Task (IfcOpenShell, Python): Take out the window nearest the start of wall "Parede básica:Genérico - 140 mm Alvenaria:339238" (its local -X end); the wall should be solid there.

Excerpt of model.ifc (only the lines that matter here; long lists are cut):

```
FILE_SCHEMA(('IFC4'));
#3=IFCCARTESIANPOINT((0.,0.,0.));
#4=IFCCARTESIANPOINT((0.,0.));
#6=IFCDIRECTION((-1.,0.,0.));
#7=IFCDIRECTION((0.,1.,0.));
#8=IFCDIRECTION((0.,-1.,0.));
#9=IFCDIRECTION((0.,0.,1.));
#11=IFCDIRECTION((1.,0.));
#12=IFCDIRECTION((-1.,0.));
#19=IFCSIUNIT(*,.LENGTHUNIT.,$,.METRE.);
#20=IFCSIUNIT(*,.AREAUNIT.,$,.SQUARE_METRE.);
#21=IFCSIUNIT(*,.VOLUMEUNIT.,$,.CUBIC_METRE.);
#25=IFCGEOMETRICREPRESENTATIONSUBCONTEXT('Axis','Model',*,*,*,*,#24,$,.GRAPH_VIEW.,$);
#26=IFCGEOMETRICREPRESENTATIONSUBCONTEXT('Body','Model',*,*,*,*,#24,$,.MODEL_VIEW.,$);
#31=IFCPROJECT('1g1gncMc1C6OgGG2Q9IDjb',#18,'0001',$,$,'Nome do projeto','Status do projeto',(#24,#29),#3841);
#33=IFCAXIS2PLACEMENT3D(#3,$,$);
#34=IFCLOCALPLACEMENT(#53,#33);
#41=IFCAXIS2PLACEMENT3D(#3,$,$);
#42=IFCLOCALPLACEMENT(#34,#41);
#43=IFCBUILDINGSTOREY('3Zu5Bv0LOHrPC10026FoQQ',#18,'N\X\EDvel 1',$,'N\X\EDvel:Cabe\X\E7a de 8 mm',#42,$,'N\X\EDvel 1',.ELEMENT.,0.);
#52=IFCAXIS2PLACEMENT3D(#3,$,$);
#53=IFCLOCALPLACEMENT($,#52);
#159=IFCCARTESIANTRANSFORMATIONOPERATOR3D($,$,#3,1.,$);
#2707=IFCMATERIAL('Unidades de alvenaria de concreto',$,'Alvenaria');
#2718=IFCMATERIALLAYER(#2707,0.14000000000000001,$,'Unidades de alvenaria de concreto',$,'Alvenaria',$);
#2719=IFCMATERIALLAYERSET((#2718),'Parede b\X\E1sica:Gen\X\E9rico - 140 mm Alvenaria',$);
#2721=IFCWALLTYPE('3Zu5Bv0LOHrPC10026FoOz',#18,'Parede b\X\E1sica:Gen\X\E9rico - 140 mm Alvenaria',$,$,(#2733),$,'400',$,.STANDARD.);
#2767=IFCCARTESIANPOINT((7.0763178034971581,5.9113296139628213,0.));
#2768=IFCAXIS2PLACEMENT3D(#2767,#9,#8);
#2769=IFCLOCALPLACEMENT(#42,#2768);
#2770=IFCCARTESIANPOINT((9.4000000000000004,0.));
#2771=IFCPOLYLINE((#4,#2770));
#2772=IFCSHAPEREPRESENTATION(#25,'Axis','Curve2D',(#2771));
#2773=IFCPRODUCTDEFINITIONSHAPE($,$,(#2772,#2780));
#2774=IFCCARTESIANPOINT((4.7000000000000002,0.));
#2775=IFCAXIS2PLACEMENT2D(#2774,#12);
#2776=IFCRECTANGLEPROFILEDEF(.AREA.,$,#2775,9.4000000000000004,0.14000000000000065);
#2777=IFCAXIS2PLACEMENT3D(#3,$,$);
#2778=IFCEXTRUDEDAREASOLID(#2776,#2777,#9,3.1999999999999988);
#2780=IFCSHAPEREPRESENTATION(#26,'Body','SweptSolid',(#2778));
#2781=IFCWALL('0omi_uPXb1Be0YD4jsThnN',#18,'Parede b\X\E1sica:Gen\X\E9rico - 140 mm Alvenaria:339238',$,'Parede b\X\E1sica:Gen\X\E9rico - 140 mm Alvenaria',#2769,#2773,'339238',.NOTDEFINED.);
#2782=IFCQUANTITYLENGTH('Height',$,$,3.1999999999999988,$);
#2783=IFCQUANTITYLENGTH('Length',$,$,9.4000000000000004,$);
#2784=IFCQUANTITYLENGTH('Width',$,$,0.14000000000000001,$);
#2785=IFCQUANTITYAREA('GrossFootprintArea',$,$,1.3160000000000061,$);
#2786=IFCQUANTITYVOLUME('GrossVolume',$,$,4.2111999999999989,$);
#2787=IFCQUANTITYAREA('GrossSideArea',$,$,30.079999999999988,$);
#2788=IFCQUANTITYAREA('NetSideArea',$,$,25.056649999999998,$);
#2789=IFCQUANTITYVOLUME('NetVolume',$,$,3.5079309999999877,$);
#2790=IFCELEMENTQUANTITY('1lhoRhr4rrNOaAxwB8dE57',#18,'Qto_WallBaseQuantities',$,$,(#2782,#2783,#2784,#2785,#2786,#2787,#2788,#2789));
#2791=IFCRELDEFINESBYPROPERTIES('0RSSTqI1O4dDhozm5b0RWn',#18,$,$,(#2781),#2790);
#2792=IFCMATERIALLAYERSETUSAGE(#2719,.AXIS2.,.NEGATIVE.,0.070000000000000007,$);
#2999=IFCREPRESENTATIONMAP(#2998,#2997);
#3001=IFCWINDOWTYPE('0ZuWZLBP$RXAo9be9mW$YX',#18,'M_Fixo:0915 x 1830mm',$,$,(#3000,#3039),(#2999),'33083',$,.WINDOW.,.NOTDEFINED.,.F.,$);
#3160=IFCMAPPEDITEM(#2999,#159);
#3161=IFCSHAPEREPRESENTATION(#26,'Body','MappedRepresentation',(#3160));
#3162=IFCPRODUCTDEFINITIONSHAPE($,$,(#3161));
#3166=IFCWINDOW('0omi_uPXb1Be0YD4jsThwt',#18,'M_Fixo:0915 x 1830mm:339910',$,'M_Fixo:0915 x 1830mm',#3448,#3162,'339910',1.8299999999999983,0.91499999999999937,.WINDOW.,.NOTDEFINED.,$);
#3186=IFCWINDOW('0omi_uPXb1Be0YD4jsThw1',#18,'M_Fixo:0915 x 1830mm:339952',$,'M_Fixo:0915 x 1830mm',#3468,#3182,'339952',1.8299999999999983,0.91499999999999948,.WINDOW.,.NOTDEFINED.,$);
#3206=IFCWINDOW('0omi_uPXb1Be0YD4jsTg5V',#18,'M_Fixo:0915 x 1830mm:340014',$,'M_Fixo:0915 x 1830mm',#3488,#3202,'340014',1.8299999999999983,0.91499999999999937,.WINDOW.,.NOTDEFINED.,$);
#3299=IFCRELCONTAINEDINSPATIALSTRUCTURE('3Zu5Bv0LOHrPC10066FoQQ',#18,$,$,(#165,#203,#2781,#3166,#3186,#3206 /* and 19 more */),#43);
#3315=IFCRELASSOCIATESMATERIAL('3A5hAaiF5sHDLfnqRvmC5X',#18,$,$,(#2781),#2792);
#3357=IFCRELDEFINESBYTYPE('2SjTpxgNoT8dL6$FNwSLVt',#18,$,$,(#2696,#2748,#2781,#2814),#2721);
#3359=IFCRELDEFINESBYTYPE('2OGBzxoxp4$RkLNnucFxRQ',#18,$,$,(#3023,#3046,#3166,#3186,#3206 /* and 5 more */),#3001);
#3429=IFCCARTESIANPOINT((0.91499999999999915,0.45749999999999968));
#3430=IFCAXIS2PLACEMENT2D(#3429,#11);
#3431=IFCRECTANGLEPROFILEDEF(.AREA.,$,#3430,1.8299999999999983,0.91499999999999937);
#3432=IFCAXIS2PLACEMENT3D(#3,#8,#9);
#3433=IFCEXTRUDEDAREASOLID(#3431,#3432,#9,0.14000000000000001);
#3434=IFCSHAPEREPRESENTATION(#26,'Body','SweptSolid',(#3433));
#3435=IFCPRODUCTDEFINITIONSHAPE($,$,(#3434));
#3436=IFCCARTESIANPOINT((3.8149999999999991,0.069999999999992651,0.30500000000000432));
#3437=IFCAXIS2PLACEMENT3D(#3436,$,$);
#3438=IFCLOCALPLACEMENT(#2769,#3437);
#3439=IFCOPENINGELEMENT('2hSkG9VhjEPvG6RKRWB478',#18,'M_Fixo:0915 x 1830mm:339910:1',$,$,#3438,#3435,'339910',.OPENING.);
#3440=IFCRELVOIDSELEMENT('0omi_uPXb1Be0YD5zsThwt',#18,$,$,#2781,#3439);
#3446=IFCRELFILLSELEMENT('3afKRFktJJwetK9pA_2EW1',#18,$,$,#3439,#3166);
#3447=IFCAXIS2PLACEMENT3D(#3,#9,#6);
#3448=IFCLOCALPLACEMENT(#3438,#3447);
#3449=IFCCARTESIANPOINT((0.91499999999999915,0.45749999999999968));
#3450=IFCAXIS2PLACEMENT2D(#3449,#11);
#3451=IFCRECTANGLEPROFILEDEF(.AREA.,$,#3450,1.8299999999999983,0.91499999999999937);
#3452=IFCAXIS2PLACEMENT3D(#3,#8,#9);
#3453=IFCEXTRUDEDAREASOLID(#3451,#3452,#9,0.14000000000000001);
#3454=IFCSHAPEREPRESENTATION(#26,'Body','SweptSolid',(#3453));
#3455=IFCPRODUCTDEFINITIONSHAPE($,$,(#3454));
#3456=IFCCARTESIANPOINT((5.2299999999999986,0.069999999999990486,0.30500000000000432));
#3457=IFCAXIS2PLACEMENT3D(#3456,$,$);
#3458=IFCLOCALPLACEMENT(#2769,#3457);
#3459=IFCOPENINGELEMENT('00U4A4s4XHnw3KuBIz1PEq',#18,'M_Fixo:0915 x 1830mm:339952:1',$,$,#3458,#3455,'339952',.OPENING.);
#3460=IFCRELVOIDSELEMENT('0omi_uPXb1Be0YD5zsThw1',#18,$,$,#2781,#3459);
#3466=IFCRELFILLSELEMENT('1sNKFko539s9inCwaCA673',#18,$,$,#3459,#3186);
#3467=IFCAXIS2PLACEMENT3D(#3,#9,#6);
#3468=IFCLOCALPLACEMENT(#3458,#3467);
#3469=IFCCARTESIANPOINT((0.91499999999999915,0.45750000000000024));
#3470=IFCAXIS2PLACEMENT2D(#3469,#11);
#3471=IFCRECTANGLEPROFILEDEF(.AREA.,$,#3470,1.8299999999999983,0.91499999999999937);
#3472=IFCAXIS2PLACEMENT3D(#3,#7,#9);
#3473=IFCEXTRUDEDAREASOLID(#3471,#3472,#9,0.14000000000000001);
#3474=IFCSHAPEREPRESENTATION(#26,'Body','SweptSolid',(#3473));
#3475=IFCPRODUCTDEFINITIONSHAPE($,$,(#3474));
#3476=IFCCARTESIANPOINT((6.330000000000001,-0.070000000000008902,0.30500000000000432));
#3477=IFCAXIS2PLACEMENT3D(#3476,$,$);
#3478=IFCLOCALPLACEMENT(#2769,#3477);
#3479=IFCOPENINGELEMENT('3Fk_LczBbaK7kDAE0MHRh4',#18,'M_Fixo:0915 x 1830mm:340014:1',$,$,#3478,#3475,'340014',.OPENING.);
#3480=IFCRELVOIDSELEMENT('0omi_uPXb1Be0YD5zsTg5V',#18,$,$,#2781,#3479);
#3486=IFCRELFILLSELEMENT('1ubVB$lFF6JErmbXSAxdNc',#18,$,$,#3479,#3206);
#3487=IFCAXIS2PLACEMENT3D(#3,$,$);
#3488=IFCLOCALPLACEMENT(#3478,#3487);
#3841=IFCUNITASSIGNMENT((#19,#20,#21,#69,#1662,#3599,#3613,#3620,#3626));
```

```python
import ifcopenshell
import ifcopenshell.api.feature
import ifcopenshell.api.pset
import ifcopenshell.api.root
import ifcopenshell.geom
import ifcopenshell.util.element
import ifcopenshell.util.shape
import ifcopenshell.util.unit

model = ifcopenshell.open("model.ifc")
area_scale = ifcopenshell.util.unit.calculate_unit_scale(model, "AREAUNIT")
volume_scale = ifcopenshell.util.unit.calculate_unit_scale(model, "VOLUMEUNIT")
settings = ifcopenshell.geom.settings()


def volume(element):
    """Net volume in cubic metres, openings subtracted."""
    shape = ifcopenshell.geom.create_shape(settings, element)
    return ifcopenshell.util.shape.get_volume(shape.geometry)


window = model.by_guid("0omi_uPXb1Be0YD4jsThwt")
opening = window.FillsVoids[0].RelatingOpeningElement
wall = opening.VoidsElements[0].RelatingBuildingElement
before = volume(wall)

ifcopenshell.api.root.remove_product(model, product=window)
ifcopenshell.api.feature.remove_feature(model, feature=opening)

after = volume(wall)
thickness = 0.14  # wall thickness in metres

# Update the wall's stored quantities.
qto = model.by_id(ifcopenshell.util.element.get_pset(wall, "Qto_WallBaseQuantities", should_inherit=False)["id"])
ifcopenshell.api.pset.edit_qto(model, qto=qto, properties={
    "NetSideArea": after / thickness / area_scale,
    "NetVolume": after / volume_scale,
})

print(f"wall volume {before:.3f} -> {after:.3f} m3")

model.write("model_edited.ifc")
```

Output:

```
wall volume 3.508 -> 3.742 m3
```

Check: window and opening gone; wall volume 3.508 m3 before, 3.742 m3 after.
